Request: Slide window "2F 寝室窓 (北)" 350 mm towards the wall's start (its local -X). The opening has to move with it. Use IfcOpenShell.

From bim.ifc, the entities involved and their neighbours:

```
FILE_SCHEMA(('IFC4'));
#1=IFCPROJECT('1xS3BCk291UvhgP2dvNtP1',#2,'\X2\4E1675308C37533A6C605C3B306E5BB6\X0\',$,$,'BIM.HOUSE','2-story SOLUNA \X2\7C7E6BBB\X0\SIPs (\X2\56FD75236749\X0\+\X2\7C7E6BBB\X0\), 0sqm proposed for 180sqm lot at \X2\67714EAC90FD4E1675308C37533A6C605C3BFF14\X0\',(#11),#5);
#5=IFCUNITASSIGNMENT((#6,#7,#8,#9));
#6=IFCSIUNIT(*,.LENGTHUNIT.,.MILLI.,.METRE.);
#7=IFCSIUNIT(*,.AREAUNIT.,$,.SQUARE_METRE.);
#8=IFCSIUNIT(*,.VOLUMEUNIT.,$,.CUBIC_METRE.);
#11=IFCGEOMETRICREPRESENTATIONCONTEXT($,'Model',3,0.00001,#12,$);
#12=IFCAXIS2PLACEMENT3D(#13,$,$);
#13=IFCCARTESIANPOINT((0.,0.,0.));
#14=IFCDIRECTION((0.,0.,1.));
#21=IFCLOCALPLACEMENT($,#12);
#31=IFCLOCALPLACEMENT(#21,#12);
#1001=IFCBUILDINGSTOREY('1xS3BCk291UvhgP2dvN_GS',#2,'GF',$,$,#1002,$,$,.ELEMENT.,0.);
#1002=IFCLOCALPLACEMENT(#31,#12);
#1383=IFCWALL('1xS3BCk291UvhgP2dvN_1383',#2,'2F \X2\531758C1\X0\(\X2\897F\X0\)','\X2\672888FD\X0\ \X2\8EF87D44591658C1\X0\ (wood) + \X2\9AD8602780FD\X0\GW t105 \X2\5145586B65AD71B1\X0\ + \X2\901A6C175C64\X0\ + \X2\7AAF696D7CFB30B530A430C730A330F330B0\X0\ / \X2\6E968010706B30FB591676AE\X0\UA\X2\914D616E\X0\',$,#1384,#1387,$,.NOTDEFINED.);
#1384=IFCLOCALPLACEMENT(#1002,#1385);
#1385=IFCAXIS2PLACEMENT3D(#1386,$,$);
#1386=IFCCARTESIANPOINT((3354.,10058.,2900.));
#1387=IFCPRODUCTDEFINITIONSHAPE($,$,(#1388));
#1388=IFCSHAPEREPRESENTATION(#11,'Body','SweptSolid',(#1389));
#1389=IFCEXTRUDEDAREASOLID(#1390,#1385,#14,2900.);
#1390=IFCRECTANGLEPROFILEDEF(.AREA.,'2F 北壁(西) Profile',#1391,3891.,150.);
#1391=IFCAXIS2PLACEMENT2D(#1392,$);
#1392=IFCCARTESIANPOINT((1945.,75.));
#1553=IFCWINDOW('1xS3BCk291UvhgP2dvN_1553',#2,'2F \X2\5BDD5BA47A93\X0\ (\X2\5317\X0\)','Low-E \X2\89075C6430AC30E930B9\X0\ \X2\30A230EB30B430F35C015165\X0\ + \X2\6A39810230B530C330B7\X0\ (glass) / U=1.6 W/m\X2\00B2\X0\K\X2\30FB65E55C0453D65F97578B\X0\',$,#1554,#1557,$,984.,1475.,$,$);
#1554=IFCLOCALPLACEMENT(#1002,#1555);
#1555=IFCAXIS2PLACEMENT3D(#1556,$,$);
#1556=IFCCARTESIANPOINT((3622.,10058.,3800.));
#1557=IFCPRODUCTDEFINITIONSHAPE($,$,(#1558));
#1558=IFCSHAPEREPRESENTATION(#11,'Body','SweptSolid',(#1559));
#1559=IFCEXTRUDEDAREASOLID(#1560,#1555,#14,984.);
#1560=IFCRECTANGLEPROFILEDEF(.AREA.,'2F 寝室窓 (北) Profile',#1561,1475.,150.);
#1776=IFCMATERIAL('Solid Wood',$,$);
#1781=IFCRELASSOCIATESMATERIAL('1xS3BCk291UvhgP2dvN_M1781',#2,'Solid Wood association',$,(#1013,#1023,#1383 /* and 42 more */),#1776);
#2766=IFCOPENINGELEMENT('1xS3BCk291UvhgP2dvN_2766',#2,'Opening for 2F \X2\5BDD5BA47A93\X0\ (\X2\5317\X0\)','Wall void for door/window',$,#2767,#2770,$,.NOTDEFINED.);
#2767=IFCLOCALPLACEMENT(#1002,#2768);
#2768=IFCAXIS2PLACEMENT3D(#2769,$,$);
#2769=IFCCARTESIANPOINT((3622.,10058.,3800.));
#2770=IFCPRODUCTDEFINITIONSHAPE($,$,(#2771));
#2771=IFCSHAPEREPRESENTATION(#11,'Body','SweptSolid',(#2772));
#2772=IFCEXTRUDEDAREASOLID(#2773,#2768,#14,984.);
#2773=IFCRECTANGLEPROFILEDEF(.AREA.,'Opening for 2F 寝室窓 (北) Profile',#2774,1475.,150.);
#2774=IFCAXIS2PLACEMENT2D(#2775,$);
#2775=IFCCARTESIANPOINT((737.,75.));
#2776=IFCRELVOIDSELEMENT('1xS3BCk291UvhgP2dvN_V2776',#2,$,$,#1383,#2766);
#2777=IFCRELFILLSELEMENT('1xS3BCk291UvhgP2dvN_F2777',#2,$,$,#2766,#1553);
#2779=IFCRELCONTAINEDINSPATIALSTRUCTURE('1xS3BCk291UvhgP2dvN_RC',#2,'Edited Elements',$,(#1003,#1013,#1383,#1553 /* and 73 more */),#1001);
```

```python
import ifcopenshell
import ifcopenshell.api.geometry
import ifcopenshell.util.placement
import ifcopenshell.util.unit

model = ifcopenshell.open("bim.ifc")
unit_scale = ifcopenshell.util.unit.calculate_unit_scale(model)

window = model.by_id(1553)
opening = window.FillsVoids[0].RelatingOpeningElement
wall = opening.VoidsElements[0].RelatingBuildingElement

wall_matrix = ifcopenshell.util.placement.get_local_placement(wall.ObjectPlacement)
shift = wall_matrix[:3, 0] * -0.35 / unit_scale
before = ifcopenshell.util.placement.get_local_placement(window.ObjectPlacement)[:3, 3].copy()

# The window is not placed relative to its opening, so move both.
for product in (opening, window):
    matrix = ifcopenshell.util.placement.get_local_placement(product.ObjectPlacement)
    matrix[:3, 3] += shift
    ifcopenshell.api.geometry.edit_object_placement(model, product=product, matrix=matrix, is_si=False)

after = ifcopenshell.util.placement.get_local_placement(window.ObjectPlacement)[:3, 3]
print("window moved by", (after - before).round(3) + 0.0)

model.write("bim_edited.ifc")
```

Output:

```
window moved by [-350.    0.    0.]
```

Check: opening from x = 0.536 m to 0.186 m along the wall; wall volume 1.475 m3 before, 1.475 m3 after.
